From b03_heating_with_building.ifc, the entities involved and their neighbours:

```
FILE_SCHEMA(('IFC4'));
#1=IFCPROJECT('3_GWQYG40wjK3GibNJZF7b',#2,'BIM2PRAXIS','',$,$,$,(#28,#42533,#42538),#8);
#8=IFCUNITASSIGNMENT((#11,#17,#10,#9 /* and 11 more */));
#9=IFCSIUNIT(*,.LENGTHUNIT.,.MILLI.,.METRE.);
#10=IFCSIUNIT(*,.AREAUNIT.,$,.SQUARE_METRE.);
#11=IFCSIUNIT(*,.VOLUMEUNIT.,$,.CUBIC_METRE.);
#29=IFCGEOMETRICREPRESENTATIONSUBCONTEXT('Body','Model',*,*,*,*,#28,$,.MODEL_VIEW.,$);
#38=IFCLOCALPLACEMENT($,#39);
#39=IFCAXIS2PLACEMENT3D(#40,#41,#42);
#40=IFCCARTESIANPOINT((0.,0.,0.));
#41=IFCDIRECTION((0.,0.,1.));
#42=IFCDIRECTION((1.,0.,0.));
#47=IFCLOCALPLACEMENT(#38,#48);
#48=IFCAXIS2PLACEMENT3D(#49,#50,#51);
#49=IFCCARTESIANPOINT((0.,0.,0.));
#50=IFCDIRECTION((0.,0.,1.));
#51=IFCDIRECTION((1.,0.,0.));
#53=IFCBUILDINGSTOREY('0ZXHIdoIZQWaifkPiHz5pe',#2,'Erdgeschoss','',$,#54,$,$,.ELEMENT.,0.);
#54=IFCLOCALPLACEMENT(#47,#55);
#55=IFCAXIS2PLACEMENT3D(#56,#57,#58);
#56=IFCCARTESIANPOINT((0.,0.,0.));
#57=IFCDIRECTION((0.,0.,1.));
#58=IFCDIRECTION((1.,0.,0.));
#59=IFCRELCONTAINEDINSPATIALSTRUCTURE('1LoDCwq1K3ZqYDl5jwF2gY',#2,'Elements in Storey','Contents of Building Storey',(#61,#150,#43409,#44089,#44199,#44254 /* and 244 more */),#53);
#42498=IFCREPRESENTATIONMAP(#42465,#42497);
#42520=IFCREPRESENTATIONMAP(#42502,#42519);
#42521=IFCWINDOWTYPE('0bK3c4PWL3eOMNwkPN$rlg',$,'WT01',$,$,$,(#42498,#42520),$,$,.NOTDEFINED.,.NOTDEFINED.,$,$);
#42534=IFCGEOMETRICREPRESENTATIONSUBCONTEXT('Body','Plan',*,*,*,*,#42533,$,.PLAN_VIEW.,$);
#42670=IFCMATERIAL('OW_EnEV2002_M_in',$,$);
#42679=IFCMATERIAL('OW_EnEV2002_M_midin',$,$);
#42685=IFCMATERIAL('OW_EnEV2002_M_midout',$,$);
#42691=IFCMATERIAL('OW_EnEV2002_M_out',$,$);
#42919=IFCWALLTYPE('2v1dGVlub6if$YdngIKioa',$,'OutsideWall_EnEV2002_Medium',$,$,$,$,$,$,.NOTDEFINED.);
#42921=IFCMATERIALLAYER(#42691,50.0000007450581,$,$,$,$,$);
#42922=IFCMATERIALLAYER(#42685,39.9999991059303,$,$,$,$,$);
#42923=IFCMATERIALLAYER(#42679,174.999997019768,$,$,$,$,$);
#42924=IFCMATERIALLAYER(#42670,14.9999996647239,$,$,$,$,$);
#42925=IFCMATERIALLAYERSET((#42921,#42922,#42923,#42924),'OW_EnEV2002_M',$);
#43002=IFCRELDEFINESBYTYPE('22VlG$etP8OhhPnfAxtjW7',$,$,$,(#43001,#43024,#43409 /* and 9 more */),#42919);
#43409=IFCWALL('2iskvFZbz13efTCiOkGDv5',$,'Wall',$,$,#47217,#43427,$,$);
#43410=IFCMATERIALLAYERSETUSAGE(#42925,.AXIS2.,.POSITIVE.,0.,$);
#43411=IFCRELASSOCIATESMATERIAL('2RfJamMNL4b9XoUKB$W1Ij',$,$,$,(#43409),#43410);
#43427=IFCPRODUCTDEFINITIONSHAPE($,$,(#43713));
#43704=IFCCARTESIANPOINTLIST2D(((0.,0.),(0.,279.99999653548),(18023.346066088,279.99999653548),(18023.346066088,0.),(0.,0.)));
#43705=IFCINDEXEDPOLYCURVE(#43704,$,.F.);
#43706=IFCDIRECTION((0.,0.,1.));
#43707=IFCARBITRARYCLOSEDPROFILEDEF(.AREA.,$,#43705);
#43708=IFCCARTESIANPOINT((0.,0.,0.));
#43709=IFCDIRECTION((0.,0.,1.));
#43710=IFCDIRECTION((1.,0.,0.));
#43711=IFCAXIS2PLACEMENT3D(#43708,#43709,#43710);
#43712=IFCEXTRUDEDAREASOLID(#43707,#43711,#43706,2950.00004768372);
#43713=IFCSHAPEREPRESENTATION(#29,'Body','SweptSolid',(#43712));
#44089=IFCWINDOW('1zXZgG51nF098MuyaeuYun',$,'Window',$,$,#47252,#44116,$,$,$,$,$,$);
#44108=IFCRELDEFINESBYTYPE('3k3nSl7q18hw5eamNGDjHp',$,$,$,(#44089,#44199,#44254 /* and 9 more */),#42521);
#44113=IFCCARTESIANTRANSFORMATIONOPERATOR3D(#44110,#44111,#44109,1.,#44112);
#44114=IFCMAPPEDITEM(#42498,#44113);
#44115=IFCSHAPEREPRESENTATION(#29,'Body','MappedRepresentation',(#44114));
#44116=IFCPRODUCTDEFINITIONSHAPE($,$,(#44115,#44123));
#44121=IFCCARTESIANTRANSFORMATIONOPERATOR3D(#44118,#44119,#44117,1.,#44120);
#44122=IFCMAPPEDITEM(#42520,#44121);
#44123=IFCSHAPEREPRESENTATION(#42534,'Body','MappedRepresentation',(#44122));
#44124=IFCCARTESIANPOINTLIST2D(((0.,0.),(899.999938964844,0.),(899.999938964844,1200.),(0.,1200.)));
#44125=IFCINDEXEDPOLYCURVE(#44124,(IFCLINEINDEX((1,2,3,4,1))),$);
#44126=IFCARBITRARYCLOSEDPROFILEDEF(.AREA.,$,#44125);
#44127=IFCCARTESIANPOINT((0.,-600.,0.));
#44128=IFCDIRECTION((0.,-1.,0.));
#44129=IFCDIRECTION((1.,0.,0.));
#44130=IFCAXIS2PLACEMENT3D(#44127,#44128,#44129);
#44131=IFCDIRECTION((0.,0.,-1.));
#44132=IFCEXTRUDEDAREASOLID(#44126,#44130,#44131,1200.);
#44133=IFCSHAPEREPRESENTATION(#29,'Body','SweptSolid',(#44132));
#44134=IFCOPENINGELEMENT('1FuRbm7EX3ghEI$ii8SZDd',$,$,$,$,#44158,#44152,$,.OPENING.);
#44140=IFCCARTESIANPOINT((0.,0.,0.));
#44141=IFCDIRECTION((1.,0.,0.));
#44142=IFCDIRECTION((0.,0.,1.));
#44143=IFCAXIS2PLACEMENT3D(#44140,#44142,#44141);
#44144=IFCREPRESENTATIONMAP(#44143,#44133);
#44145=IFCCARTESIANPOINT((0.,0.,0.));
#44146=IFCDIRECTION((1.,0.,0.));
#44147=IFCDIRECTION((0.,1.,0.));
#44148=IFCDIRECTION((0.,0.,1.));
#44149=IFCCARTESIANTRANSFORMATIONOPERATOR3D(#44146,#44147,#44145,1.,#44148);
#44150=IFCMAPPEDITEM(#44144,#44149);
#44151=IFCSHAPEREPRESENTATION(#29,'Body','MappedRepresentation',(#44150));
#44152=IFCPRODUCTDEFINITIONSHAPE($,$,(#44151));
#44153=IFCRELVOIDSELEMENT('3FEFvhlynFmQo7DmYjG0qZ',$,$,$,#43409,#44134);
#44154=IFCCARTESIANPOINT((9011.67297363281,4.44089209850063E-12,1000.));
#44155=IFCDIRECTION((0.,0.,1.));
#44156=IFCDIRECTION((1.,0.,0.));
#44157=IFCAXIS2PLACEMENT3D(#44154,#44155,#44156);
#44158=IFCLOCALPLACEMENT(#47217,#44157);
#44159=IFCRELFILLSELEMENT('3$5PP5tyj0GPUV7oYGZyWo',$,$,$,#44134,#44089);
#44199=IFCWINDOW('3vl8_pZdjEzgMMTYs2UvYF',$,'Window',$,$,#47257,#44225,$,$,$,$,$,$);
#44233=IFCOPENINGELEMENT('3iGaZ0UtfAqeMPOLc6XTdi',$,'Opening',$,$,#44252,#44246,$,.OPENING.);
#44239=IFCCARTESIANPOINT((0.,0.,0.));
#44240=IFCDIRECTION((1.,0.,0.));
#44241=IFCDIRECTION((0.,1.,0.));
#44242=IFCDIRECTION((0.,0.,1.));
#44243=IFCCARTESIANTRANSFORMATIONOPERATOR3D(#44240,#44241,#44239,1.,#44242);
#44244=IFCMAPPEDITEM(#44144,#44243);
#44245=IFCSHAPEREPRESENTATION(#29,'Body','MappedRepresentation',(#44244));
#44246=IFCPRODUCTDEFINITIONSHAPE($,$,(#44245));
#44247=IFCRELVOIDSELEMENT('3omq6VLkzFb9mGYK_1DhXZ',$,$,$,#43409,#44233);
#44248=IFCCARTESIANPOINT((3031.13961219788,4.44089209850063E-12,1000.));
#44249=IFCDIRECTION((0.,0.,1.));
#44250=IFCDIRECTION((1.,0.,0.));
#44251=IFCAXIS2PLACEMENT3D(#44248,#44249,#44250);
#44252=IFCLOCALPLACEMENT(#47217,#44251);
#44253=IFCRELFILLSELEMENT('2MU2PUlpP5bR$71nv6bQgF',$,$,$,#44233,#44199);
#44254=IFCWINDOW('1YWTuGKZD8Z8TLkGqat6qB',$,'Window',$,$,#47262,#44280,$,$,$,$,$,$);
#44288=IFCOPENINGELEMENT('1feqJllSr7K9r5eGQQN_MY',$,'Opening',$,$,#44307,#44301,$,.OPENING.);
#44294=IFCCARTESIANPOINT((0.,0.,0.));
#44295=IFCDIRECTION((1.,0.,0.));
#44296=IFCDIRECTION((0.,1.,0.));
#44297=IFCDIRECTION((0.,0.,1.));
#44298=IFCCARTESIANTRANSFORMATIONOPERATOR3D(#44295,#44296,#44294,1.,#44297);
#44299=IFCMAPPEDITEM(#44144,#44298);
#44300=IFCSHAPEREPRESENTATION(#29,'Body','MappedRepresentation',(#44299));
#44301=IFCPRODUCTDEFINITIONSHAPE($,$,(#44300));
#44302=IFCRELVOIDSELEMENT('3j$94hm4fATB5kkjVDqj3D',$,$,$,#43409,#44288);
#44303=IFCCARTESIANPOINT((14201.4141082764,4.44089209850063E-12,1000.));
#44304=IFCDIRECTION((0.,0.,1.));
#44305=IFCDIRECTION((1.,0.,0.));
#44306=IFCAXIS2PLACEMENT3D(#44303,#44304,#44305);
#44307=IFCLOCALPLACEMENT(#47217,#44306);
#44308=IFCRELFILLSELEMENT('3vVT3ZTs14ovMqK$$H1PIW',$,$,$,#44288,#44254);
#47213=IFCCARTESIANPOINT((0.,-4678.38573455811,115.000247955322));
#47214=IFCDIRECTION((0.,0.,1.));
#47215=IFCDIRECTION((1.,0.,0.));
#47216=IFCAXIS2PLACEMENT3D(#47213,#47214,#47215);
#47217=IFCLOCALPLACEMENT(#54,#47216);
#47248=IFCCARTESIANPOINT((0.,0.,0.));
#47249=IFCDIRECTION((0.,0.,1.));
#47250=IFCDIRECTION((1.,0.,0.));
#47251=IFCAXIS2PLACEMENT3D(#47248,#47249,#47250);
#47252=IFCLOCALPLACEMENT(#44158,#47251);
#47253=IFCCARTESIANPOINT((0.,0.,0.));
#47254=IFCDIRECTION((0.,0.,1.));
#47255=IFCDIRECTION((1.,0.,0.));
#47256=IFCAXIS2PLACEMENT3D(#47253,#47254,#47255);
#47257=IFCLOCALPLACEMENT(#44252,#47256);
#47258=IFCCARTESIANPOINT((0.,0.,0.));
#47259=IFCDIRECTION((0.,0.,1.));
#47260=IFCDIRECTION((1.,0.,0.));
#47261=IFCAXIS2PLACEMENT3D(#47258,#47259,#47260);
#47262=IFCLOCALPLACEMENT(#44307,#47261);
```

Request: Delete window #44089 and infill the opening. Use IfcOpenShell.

```python
import ifcopenshell
import ifcopenshell.api.feature
import ifcopenshell.api.root
import ifcopenshell.geom
import ifcopenshell.util.shape

model = ifcopenshell.open("b03_heating_with_building.ifc")
settings = ifcopenshell.geom.settings()


def volume(element):
    """Net volume in cubic metres, openings subtracted."""
    shape = ifcopenshell.geom.create_shape(settings, element)
    return ifcopenshell.util.shape.get_volume(shape.geometry)


window = model.by_id(44089)
opening = window.FillsVoids[0].RelatingOpeningElement
wall = opening.VoidsElements[0].RelatingBuildingElement
before = volume(wall)

ifcopenshell.api.root.remove_product(model, product=window)
ifcopenshell.api.feature.remove_feature(model, feature=opening)

after = volume(wall)

print(f"wall volume {before:.3f} -> {after:.3f} m3")

model.write("b03_heating_with_building_updated.ifc")
```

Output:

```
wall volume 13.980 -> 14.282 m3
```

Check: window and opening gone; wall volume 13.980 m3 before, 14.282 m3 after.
